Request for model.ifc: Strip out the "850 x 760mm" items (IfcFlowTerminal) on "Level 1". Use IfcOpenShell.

First a look at what the model holds.

```python
import ifcopenshell
import ifcopenshell.util.element

model = ifcopenshell.open("model.ifc")
print(model.schema)
storey = next(s for s in model.by_type("IfcBuildingStorey") if s.Name == "Level 1")
terminals = [e for e in ifcopenshell.util.element.get_decomposition(storey) if e.is_a("IfcFlowTerminal")]
seen = {}
for e in terminals:
    element_type = ifcopenshell.util.element.get_type(e)
    name = element_type.Name if element_type not in (None, e) else None
    seen[name] = seen.get(name, 0) + 1
for name, count in sorted(seen.items(), key=str):
    print(count, "x", name)
```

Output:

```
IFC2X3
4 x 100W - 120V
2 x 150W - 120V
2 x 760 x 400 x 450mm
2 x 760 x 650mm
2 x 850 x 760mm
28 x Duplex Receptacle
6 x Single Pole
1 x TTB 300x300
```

```python
import ifcopenshell
import ifcopenshell.api.root
import ifcopenshell.util.element

model = ifcopenshell.open("model.ifc")

storey = next(s for s in model.by_type("IfcBuildingStorey") if s.Name == "Level 1")
terminals = [e for e in ifcopenshell.util.element.get_decomposition(storey) if e.is_a("IfcFlowTerminal")]
targets = [e for e in terminals if (t := ifcopenshell.util.element.get_type(e)) not in (None, e) and t.Name == "850 x 760mm"]

for e in targets:
    ifcopenshell.api.root.remove_product(model, product=e)
print(len(targets), "removed")

model.write("model_v2.ifc")
```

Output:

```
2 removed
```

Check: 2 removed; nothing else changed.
